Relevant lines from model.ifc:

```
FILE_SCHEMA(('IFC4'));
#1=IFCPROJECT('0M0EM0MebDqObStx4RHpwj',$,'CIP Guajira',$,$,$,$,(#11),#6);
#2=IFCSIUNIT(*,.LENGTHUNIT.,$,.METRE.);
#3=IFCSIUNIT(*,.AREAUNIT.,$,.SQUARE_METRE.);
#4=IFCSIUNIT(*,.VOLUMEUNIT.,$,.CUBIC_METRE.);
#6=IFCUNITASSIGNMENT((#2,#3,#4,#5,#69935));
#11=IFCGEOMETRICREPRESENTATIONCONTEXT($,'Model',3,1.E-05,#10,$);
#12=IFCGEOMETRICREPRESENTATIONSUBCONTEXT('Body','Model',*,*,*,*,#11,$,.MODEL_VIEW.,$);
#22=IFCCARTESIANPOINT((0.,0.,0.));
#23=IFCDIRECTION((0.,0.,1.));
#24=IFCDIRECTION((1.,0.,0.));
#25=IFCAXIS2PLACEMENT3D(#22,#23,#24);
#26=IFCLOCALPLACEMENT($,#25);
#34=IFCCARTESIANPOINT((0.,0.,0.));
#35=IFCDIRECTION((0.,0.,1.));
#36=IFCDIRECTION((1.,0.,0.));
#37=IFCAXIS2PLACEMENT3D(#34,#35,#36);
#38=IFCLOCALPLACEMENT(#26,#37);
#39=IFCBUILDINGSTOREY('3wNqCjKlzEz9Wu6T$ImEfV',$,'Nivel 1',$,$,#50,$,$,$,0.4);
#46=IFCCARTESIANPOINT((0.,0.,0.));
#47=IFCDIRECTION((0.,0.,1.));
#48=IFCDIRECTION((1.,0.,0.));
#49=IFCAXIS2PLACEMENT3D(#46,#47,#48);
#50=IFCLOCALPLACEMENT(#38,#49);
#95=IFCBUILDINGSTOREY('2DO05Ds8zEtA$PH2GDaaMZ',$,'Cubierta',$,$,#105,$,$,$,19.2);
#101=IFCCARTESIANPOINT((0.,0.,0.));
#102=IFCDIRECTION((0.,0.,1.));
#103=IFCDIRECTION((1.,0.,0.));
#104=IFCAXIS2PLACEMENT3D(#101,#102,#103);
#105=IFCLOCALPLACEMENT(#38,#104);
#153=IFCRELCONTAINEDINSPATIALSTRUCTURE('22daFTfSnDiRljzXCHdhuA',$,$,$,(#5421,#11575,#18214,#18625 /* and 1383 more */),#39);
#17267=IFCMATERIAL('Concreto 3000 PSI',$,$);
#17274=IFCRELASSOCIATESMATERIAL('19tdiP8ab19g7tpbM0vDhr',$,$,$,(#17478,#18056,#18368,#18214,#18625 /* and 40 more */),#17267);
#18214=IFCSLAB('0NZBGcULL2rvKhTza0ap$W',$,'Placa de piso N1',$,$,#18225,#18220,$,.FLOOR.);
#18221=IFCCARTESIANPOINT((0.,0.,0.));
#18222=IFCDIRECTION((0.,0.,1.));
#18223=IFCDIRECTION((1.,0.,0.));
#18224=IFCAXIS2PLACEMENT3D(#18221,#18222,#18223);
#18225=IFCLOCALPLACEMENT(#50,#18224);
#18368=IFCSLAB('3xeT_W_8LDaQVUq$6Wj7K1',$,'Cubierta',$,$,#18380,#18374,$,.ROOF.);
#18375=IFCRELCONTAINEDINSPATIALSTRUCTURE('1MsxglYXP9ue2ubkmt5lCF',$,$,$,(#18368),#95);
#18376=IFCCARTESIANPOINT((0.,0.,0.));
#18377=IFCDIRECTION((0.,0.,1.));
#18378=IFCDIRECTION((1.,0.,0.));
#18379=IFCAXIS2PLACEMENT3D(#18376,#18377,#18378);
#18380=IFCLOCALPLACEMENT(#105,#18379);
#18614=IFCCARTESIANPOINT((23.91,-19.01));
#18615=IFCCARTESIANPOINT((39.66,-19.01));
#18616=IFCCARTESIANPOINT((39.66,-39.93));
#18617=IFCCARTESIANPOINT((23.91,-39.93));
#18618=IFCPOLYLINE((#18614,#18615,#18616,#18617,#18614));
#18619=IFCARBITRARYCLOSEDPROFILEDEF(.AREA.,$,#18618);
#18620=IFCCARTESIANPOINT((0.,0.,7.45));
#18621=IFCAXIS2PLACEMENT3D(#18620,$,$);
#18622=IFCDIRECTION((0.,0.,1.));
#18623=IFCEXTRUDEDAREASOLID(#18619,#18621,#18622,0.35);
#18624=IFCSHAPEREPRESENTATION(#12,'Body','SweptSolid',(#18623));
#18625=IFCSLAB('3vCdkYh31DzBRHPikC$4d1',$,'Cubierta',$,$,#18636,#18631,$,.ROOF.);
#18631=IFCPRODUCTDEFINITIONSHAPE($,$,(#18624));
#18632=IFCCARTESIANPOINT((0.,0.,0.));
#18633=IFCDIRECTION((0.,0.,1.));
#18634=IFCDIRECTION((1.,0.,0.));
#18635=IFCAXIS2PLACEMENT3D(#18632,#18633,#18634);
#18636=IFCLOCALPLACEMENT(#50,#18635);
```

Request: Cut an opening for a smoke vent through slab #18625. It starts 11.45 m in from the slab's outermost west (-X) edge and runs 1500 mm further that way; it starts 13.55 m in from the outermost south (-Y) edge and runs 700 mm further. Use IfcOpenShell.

```python
import numpy as np
import ifcopenshell
import ifcopenshell.api.feature
import ifcopenshell.api.geometry
import ifcopenshell.api.root
import ifcopenshell.geom
import ifcopenshell.util.placement
import ifcopenshell.util.representation
import ifcopenshell.util.shape
import ifcopenshell.util.unit

model = ifcopenshell.open("model.ifc")
unit_scale = ifcopenshell.util.unit.calculate_unit_scale(model)
settings = ifcopenshell.geom.settings()


def volume(element):
    """Net volume in cubic metres, openings subtracted."""
    shape = ifcopenshell.geom.create_shape(settings, element)
    return ifcopenshell.util.shape.get_volume(shape.geometry)


slab = model.by_guid("3vCdkYh31DzBRHPikC$4d1")
before = volume(slab)

# Extent in the slab's own axes, in metres. The edges named are its -X and -Y sides.
slab_shape = ifcopenshell.geom.create_shape(settings, slab)
vertices = ifcopenshell.util.shape.get_vertices(slab_shape.geometry)
x_min, y_min, bottom = vertices.min(axis=0)
top = vertices[:, 2].max()

opening = ifcopenshell.api.root.create_entity(model, ifc_class="IfcOpeningElement", name="Smoke vent opening", predefined_type="OPENING")
context = ifcopenshell.util.representation.get_context(model, "Model", "Body", "MODEL_VIEW")
width, depth = 1.5, 0.7
outline = [(0.0, 0.0), (width, 0.0), (width, depth), (0.0, depth), (0.0, 0.0)]
# Overshoot both faces by 50 mm so the cut is clean.
shape = ifcopenshell.api.geometry.add_slab_representation(
    model, context=context, depth=top - bottom + 0.1, polyline=outline
)
ifcopenshell.api.geometry.assign_representation(model, product=opening, representation=shape)

matrix = ifcopenshell.util.placement.get_local_placement(slab.ObjectPlacement)
matrix[:, 3] = matrix @ np.append(np.array([x_min + 11.45, y_min + 13.55, bottom - 0.05]) / unit_scale, 1.0)
ifcopenshell.api.geometry.edit_object_placement(model, product=opening, matrix=matrix, is_si=False)
ifcopenshell.api.feature.add_feature(model, feature=opening, element=slab)

after = volume(slab)

print(f"slab volume {before:.3f} -> {after:.3f} m3")

model.write("model_edited.ifc")
```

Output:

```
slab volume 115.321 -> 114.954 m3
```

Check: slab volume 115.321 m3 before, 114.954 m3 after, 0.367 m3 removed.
